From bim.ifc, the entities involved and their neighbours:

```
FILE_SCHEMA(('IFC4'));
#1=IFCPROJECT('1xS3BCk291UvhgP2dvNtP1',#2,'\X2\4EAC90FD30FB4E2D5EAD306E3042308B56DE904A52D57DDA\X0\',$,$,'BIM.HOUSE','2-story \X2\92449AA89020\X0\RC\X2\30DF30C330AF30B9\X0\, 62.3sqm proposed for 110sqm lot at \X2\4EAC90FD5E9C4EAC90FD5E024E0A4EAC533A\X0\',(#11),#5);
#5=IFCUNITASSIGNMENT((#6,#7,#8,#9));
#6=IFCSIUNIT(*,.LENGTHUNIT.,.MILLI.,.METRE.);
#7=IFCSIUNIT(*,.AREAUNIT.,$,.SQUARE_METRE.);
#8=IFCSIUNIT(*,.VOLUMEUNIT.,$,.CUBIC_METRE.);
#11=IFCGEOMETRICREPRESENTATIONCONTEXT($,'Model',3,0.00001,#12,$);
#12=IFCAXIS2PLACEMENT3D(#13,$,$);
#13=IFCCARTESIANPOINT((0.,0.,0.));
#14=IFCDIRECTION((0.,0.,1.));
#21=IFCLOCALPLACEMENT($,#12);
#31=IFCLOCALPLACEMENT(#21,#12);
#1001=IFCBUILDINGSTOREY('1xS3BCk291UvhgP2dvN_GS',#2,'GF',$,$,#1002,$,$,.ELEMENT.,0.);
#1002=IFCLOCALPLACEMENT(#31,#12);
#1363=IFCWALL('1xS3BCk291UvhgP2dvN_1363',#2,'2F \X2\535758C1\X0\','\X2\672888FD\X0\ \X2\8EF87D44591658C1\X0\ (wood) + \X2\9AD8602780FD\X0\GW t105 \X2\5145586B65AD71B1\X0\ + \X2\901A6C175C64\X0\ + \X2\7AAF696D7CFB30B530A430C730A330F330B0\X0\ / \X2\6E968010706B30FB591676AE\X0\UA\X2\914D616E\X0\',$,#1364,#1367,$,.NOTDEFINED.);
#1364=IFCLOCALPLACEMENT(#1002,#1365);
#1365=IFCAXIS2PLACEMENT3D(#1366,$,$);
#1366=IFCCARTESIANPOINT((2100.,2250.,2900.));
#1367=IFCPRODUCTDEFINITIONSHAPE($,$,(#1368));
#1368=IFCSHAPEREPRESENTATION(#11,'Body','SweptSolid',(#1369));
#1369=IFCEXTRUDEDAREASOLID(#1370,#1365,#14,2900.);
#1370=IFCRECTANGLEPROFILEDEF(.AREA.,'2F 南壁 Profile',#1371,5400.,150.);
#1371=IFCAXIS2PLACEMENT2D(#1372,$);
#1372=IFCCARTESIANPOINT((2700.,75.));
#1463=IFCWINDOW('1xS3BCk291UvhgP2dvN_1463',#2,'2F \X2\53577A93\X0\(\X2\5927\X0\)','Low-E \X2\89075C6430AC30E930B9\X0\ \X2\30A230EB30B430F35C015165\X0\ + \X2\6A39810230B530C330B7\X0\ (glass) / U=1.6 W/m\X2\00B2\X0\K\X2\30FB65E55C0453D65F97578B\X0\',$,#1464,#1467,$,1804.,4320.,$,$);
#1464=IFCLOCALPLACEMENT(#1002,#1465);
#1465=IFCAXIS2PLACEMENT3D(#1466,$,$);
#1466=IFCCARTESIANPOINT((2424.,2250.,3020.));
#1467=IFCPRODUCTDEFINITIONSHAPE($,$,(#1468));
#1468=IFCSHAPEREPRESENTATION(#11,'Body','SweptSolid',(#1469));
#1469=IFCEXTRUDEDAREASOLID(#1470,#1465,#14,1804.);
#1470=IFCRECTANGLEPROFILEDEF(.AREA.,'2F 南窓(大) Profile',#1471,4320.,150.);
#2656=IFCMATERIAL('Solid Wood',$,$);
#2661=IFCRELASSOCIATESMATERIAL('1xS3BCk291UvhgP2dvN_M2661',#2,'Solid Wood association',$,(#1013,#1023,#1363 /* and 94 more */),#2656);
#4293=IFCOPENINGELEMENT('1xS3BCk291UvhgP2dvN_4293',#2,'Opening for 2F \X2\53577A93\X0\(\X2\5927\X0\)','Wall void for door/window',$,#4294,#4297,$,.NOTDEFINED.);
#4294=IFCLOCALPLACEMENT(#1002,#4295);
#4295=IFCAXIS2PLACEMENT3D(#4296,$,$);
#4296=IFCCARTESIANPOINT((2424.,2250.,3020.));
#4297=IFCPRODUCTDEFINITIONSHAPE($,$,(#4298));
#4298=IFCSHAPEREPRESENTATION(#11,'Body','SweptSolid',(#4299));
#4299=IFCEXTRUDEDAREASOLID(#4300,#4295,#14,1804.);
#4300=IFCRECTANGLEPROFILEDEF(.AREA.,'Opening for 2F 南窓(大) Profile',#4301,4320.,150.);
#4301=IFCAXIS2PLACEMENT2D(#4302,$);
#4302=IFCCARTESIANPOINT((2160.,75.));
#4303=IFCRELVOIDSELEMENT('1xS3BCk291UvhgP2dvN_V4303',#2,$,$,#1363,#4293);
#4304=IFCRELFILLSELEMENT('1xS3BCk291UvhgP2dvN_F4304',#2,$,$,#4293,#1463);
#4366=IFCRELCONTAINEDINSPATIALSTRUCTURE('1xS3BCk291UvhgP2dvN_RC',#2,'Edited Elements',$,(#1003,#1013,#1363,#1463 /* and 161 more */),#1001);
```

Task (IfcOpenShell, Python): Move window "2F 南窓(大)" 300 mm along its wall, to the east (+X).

```python
import ifcopenshell
import ifcopenshell.api.geometry
import ifcopenshell.util.placement

model = ifcopenshell.open("bim.ifc")

window = model.by_guid("1xS3BCk291UvhgP2dvN_1463")
opening = window.FillsVoids[0].RelatingOpeningElement
wall = opening.VoidsElements[0].RelatingBuildingElement

wall_matrix = ifcopenshell.util.placement.get_local_placement(wall.ObjectPlacement)
shift = wall_matrix[:3, 0] * 300.0
before = ifcopenshell.util.placement.get_local_placement(window.ObjectPlacement)[:3, 3].copy()

# The window is not placed relative to its opening, so move both.
for product in (opening, window):
    matrix = ifcopenshell.util.placement.get_local_placement(product.ObjectPlacement)
    matrix[:3, 3] += shift
    ifcopenshell.api.geometry.edit_object_placement(model, product=product, matrix=matrix, is_si=False)

after = ifcopenshell.util.placement.get_local_placement(window.ObjectPlacement)[:3, 3]
print("window moved by", (after - before).round(3) + 0.0)

model.write("bim-out.ifc")
```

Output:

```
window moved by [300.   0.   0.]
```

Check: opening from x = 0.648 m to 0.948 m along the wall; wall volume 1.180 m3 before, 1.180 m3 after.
